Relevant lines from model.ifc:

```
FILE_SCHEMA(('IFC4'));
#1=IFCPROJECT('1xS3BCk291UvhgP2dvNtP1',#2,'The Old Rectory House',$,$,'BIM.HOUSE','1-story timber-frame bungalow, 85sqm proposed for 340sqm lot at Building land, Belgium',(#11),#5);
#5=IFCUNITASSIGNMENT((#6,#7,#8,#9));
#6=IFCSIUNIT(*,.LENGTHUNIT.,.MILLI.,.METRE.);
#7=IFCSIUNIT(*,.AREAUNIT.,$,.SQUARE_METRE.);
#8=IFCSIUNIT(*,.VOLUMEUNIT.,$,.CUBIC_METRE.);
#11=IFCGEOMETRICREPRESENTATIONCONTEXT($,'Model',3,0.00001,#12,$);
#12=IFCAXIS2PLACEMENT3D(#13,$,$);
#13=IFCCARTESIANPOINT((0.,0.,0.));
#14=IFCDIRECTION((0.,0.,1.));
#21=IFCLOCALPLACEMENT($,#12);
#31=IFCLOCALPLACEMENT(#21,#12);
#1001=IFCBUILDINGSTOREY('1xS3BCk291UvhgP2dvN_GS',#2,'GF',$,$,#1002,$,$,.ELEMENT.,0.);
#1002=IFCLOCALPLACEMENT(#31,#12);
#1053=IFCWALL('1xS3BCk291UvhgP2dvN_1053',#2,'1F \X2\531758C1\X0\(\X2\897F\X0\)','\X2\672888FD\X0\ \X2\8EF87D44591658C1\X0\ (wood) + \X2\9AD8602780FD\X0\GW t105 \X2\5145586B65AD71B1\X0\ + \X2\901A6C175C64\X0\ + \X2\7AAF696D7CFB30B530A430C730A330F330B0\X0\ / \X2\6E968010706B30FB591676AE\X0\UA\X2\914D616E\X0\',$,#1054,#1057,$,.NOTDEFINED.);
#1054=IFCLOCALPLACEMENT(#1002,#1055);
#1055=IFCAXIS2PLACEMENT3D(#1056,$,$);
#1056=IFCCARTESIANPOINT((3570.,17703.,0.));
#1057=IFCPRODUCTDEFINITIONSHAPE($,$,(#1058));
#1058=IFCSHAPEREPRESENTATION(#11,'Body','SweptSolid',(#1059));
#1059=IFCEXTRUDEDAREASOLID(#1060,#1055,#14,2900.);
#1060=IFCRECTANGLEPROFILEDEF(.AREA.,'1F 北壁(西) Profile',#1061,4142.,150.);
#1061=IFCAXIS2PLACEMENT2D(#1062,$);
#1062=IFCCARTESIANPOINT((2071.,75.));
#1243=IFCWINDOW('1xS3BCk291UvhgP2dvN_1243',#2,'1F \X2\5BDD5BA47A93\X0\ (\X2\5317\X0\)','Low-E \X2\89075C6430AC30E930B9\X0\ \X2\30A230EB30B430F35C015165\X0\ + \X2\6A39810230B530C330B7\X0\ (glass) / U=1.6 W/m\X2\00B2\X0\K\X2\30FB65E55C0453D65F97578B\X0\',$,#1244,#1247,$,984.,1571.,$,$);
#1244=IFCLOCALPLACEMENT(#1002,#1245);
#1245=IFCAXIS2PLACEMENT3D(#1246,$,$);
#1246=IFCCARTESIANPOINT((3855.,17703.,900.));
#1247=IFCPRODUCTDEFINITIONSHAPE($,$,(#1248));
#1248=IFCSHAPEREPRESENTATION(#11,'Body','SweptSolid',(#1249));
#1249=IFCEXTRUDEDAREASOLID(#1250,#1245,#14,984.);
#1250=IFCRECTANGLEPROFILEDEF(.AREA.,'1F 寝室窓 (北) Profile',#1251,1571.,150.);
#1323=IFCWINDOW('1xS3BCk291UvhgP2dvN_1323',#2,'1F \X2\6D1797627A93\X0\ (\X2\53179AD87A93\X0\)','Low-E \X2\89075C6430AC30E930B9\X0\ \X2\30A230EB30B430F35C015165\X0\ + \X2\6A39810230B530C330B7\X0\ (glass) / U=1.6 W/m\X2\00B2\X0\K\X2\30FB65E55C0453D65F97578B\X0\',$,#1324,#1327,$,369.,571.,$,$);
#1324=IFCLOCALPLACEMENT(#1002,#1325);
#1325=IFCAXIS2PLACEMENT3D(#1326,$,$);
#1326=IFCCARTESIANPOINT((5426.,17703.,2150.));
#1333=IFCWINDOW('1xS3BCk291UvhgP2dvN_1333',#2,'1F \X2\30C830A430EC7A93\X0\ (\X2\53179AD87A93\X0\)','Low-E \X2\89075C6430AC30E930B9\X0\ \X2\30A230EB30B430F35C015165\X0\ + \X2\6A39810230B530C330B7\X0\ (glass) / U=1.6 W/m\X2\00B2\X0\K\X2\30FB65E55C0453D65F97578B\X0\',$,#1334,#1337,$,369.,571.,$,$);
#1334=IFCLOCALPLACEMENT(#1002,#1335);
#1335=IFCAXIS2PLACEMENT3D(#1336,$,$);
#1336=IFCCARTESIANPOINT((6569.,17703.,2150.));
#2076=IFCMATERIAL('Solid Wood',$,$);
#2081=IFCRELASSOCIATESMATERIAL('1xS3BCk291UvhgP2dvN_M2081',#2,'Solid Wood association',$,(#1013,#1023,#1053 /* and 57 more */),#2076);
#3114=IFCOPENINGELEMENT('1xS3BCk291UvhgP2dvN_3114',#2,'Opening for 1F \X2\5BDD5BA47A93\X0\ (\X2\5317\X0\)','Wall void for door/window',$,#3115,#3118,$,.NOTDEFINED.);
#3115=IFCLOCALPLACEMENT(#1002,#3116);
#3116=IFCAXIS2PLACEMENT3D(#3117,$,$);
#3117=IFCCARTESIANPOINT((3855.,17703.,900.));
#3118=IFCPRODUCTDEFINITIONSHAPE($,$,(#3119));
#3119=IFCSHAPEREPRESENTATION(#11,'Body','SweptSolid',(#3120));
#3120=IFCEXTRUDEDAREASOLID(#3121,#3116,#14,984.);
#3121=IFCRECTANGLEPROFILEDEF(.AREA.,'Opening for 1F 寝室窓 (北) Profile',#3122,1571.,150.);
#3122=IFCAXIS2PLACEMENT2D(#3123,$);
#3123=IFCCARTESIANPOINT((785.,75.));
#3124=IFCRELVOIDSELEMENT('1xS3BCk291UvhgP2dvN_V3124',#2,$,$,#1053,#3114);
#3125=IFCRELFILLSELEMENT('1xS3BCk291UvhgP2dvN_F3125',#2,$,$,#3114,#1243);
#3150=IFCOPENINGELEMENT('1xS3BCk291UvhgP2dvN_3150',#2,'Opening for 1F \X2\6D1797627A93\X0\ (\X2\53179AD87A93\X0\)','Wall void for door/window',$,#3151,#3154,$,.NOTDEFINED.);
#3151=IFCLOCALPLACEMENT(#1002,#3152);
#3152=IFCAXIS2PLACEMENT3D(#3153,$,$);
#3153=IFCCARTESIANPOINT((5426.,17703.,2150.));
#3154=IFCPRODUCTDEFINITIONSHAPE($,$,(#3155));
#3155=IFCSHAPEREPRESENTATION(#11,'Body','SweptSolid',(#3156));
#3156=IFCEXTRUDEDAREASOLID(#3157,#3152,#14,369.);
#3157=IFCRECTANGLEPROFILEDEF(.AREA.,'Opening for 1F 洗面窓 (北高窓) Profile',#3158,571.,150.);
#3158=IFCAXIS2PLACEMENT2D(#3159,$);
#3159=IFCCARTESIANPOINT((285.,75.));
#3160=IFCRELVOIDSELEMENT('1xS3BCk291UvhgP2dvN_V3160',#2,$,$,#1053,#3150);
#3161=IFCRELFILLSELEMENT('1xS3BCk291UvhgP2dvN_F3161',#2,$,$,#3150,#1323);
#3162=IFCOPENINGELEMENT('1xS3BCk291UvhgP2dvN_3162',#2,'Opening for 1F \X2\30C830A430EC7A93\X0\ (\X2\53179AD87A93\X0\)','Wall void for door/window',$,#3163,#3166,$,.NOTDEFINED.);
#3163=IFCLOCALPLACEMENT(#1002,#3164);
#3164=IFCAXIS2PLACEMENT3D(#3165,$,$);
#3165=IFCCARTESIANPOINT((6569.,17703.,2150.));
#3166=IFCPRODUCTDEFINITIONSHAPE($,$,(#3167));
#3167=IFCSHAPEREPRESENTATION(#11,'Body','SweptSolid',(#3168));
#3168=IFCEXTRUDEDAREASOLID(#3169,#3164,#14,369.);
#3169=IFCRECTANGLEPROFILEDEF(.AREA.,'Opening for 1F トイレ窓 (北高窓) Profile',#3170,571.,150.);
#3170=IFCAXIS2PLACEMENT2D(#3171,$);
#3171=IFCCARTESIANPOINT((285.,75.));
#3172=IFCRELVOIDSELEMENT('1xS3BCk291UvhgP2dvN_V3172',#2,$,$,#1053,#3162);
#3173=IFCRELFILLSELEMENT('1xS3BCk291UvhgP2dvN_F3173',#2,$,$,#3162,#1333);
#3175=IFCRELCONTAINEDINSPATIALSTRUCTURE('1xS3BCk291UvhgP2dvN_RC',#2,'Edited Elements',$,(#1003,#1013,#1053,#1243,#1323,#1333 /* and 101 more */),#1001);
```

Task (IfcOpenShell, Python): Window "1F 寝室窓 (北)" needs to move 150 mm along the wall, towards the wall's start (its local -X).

```python
import ifcopenshell
import ifcopenshell.api.geometry
import ifcopenshell.util.placement

model = ifcopenshell.open("model.ifc")

window = model.by_guid("1xS3BCk291UvhgP2dvN_1243")
opening = window.FillsVoids[0].RelatingOpeningElement
wall = opening.VoidsElements[0].RelatingBuildingElement

wall_matrix = ifcopenshell.util.placement.get_local_placement(wall.ObjectPlacement)
shift = wall_matrix[:3, 0] * -150.0
before = ifcopenshell.util.placement.get_local_placement(window.ObjectPlacement)[:3, 3].copy()

# The window is not placed relative to its opening, so move both.
for product in (opening, window):
    matrix = ifcopenshell.util.placement.get_local_placement(product.ObjectPlacement)
    matrix[:3, 3] += shift
    ifcopenshell.api.geometry.edit_object_placement(model, product=product, matrix=matrix, is_si=False)

after = ifcopenshell.util.placement.get_local_placement(window.ObjectPlacement)[:3, 3]
print("window moved by", (after - before).round(3) + 0.0)

model.write("model_v2.ifc")
```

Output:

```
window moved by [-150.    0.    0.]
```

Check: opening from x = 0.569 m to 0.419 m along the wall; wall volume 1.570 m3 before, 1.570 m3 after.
